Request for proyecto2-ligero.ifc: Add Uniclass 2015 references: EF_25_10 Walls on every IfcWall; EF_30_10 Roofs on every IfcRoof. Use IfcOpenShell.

First a look at what the model holds.

```python
import ifcopenshell

model = ifcopenshell.open("proyecto2-ligero.ifc")
print(model.schema)
print("classifications:", [c.Name for c in model.by_type("IfcClassification")])
for ifc_class in ("IfcDoor", "IfcRoof", "IfcStair", "IfcWall", "IfcWindow"):
    print(ifc_class, len(model.by_type(ifc_class)))
```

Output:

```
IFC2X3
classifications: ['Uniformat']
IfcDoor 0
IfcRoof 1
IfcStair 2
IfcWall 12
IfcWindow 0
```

```python
import ifcopenshell
import ifcopenshell.api.classification

model = ifcopenshell.open("proyecto2-ligero.ifc")

# IFC2X3 requires Source and Edition and has no link from the project to the system.
system = model.create_entity("IfcClassification", Source="NBS", Edition="2015", Name="Uniclass 2015")

codes = {
    "IfcWall": ("EF_25_10", "Walls"),
    "IfcRoof": ("EF_30_10", "Roofs"),
}
for ifc_class, (code, name) in codes.items():
    products = model.by_type(ifc_class)
    ifcopenshell.api.classification.add_reference(
        model, products=products, classification=system, identification=code, name=name
    )
    print(code, len(products))

model.write("proyecto2-ligero-out.ifc")
```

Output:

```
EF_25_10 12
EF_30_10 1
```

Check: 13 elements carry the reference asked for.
